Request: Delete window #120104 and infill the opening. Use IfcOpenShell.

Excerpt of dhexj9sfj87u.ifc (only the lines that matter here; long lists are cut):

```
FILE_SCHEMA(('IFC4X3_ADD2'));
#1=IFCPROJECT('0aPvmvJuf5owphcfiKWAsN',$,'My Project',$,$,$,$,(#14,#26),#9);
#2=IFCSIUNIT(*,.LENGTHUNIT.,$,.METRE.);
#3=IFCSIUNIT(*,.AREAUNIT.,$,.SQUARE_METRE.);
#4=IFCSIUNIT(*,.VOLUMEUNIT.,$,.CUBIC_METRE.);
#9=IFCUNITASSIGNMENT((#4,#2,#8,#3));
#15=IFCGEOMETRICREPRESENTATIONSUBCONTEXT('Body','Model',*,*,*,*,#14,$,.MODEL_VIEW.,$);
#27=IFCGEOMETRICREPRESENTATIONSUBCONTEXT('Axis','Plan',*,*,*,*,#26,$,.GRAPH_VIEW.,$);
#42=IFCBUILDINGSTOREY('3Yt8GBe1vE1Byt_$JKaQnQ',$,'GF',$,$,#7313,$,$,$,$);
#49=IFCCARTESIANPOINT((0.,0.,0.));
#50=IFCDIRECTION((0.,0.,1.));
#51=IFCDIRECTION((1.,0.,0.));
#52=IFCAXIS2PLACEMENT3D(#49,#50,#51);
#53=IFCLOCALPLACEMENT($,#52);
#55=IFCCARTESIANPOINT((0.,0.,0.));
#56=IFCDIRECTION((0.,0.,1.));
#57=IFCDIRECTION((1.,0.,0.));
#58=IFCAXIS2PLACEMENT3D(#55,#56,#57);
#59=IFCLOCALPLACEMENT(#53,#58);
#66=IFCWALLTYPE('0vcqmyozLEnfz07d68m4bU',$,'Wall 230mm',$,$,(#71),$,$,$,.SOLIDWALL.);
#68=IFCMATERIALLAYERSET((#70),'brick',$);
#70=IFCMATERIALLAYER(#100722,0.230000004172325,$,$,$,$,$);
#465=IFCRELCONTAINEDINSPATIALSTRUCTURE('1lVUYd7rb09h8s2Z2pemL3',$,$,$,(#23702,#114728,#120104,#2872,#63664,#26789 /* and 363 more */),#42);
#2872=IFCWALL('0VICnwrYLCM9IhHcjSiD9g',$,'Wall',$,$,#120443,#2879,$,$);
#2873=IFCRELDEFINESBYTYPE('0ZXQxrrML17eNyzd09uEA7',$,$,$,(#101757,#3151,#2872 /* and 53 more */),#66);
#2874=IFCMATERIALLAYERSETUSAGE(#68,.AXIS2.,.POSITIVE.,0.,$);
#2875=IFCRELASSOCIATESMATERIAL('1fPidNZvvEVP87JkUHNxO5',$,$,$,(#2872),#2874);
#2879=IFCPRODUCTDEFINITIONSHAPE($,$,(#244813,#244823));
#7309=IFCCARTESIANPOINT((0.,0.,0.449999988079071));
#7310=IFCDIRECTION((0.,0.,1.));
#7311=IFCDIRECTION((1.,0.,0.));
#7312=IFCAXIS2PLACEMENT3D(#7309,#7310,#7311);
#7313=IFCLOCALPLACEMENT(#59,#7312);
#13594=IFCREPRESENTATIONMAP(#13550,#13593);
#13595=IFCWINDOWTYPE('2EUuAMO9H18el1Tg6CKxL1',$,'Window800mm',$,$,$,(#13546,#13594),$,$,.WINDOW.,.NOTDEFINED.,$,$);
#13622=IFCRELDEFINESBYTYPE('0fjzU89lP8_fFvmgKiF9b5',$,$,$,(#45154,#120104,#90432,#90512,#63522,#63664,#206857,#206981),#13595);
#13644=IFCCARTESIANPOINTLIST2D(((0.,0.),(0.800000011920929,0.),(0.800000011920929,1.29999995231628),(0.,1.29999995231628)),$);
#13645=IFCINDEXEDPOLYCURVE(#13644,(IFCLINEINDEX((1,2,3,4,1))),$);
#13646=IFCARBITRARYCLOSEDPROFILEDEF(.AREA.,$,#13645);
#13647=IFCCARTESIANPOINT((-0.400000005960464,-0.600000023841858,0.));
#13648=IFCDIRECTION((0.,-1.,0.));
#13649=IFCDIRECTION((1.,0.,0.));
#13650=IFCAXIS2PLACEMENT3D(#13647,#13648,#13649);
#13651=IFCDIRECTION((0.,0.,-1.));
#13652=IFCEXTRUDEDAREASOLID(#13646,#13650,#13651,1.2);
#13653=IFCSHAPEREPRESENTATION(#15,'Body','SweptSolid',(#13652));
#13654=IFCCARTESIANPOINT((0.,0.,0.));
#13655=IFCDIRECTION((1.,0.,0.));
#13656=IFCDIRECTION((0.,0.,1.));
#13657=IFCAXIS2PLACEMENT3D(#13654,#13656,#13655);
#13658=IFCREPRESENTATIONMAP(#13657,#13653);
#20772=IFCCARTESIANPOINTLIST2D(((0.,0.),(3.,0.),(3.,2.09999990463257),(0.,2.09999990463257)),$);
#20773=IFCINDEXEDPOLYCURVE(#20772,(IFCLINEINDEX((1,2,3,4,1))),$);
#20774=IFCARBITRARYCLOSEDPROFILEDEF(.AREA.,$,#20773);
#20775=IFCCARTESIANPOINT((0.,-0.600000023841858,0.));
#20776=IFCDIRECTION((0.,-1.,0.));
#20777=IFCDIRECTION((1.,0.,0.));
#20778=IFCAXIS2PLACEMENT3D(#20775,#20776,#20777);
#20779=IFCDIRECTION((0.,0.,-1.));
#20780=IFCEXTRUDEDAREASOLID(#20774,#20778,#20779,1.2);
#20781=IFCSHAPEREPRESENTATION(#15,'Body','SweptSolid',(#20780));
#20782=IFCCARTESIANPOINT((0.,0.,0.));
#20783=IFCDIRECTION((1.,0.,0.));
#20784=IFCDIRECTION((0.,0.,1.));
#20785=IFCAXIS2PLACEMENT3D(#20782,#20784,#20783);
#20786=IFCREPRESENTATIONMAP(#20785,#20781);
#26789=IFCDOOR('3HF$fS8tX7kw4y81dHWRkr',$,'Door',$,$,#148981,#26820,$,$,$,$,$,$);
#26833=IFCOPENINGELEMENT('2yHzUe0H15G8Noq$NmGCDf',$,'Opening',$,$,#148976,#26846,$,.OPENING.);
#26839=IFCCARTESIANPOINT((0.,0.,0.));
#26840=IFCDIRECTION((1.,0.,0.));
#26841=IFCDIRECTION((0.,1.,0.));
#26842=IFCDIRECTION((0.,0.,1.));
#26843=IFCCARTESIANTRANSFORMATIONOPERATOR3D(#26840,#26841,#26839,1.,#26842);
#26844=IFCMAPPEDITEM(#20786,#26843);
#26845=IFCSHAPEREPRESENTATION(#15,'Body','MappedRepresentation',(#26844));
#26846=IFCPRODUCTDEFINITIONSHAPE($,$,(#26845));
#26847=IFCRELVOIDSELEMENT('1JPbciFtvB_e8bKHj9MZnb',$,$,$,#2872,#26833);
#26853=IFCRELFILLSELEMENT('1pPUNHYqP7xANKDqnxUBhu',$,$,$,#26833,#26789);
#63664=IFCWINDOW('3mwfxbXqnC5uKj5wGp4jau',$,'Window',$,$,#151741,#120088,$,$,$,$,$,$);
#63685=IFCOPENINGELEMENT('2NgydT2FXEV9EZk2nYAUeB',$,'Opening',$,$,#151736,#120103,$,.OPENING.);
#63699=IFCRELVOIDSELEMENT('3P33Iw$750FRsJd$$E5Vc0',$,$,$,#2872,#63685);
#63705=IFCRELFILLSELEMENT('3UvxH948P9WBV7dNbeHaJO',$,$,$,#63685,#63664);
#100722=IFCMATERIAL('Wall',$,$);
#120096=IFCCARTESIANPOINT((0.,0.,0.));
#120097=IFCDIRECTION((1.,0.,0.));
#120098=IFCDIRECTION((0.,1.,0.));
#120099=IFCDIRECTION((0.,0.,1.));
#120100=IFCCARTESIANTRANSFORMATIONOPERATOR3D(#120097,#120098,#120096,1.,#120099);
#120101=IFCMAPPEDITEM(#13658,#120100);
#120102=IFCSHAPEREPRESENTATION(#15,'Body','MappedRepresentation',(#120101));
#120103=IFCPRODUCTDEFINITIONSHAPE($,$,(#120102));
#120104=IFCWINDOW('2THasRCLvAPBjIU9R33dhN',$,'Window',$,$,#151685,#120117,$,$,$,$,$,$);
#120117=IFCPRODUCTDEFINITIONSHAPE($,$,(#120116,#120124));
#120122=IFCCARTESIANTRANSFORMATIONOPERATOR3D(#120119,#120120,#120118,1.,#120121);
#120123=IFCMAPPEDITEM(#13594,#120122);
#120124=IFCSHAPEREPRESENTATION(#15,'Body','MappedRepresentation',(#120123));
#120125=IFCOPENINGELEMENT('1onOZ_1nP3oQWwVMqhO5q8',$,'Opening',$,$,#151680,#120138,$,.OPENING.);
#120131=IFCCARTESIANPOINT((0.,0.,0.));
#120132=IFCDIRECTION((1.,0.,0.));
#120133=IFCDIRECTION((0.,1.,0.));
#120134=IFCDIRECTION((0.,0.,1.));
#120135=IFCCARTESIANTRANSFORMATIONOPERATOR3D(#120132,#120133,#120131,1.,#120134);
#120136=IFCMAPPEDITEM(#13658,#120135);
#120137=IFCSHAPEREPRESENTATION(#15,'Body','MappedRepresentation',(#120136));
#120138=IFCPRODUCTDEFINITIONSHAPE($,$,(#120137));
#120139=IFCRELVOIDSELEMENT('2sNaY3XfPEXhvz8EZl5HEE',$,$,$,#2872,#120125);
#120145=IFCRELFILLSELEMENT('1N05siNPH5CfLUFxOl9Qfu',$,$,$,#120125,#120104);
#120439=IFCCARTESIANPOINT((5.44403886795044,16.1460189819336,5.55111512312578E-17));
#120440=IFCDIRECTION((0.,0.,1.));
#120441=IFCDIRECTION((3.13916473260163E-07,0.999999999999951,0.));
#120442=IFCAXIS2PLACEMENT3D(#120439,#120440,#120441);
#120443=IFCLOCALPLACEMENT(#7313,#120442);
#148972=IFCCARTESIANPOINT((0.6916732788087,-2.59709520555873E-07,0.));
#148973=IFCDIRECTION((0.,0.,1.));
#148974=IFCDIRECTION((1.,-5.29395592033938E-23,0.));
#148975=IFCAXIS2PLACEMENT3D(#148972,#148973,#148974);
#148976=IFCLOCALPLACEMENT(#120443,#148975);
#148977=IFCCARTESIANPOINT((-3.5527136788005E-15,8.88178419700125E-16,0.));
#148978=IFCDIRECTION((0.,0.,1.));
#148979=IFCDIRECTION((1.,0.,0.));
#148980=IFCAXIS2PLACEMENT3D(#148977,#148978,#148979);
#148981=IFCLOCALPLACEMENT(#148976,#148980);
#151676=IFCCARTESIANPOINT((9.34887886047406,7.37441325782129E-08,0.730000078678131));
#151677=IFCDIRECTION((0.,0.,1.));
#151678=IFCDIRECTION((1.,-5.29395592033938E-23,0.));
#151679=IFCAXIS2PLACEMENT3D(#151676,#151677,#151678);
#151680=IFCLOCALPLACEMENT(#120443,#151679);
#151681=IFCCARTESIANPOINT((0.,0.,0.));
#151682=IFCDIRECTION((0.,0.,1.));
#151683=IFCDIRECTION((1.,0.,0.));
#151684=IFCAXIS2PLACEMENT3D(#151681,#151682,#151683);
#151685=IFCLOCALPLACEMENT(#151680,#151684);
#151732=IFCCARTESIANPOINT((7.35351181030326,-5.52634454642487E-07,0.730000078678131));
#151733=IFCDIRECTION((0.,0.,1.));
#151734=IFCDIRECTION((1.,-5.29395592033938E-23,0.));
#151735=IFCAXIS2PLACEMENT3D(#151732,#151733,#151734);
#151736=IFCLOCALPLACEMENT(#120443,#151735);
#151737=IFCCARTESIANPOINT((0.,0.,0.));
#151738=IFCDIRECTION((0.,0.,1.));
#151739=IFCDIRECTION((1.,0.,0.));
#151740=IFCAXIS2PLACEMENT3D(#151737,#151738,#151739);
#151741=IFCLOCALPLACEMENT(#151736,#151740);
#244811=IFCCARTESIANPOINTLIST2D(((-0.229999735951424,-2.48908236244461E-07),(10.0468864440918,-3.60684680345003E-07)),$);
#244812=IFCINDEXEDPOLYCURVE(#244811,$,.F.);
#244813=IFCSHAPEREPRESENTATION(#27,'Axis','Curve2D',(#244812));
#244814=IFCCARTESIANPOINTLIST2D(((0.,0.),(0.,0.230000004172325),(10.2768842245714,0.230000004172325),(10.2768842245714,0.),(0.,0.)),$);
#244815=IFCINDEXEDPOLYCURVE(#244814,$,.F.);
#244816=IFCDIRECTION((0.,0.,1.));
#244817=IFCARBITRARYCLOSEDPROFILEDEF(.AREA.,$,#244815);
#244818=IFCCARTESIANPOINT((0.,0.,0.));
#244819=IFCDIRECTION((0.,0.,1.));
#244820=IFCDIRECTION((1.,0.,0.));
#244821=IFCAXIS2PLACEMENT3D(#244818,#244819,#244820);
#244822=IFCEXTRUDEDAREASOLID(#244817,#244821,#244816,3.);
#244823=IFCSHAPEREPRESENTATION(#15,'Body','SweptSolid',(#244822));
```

```python
import ifcopenshell
import ifcopenshell.api.feature
import ifcopenshell.api.root
import ifcopenshell.geom
import ifcopenshell.util.shape

model = ifcopenshell.open("dhexj9sfj87u.ifc")
settings = ifcopenshell.geom.settings()


def volume(element):
    """Net volume in cubic metres, openings subtracted."""
    shape = ifcopenshell.geom.create_shape(settings, element)
    return ifcopenshell.util.shape.get_volume(shape.geometry)


window = model.by_guid("2THasRCLvAPBjIU9R33dhN")
opening = window.FillsVoids[0].RelatingOpeningElement
wall = opening.VoidsElements[0].RelatingBuildingElement
before = volume(wall)

ifcopenshell.api.root.remove_product(model, product=window)
ifcopenshell.api.feature.remove_feature(model, feature=opening)

after = volume(wall)

print(f"wall volume {before:.3f} -> {after:.3f} m3")

model.write("dhexj9sfj87u_v2.ifc")
```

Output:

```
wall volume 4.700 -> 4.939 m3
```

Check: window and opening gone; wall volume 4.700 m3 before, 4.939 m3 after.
